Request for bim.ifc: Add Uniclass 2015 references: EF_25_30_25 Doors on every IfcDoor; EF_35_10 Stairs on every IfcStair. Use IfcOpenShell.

First a look at what the model holds.

```python
import ifcopenshell

model = ifcopenshell.open("bim.ifc")
print(model.schema)
print("classifications:", [c.Name for c in model.by_type("IfcClassification")])
for ifc_class in ("IfcDoor", "IfcRoof", "IfcStair", "IfcWall", "IfcWindow"):
    print(ifc_class, len(model.by_type(ifc_class)))
```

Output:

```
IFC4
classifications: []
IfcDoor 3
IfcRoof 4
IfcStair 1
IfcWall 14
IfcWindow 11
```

```python
import ifcopenshell
import ifcopenshell.api.classification

model = ifcopenshell.open("bim.ifc")

system = ifcopenshell.api.classification.add_classification(model, classification="Uniclass 2015")

codes = {
    "IfcDoor": ("EF_25_30_25", "Doors"),
    "IfcStair": ("EF_35_10", "Stairs"),
}
for ifc_class, (code, name) in codes.items():
    products = model.by_type(ifc_class)
    ifcopenshell.api.classification.add_reference(
        model, products=products, classification=system, identification=code, name=name
    )
    print(code, len(products))

model.write("bim_edited.ifc")
```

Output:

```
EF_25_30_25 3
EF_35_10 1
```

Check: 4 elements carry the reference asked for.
